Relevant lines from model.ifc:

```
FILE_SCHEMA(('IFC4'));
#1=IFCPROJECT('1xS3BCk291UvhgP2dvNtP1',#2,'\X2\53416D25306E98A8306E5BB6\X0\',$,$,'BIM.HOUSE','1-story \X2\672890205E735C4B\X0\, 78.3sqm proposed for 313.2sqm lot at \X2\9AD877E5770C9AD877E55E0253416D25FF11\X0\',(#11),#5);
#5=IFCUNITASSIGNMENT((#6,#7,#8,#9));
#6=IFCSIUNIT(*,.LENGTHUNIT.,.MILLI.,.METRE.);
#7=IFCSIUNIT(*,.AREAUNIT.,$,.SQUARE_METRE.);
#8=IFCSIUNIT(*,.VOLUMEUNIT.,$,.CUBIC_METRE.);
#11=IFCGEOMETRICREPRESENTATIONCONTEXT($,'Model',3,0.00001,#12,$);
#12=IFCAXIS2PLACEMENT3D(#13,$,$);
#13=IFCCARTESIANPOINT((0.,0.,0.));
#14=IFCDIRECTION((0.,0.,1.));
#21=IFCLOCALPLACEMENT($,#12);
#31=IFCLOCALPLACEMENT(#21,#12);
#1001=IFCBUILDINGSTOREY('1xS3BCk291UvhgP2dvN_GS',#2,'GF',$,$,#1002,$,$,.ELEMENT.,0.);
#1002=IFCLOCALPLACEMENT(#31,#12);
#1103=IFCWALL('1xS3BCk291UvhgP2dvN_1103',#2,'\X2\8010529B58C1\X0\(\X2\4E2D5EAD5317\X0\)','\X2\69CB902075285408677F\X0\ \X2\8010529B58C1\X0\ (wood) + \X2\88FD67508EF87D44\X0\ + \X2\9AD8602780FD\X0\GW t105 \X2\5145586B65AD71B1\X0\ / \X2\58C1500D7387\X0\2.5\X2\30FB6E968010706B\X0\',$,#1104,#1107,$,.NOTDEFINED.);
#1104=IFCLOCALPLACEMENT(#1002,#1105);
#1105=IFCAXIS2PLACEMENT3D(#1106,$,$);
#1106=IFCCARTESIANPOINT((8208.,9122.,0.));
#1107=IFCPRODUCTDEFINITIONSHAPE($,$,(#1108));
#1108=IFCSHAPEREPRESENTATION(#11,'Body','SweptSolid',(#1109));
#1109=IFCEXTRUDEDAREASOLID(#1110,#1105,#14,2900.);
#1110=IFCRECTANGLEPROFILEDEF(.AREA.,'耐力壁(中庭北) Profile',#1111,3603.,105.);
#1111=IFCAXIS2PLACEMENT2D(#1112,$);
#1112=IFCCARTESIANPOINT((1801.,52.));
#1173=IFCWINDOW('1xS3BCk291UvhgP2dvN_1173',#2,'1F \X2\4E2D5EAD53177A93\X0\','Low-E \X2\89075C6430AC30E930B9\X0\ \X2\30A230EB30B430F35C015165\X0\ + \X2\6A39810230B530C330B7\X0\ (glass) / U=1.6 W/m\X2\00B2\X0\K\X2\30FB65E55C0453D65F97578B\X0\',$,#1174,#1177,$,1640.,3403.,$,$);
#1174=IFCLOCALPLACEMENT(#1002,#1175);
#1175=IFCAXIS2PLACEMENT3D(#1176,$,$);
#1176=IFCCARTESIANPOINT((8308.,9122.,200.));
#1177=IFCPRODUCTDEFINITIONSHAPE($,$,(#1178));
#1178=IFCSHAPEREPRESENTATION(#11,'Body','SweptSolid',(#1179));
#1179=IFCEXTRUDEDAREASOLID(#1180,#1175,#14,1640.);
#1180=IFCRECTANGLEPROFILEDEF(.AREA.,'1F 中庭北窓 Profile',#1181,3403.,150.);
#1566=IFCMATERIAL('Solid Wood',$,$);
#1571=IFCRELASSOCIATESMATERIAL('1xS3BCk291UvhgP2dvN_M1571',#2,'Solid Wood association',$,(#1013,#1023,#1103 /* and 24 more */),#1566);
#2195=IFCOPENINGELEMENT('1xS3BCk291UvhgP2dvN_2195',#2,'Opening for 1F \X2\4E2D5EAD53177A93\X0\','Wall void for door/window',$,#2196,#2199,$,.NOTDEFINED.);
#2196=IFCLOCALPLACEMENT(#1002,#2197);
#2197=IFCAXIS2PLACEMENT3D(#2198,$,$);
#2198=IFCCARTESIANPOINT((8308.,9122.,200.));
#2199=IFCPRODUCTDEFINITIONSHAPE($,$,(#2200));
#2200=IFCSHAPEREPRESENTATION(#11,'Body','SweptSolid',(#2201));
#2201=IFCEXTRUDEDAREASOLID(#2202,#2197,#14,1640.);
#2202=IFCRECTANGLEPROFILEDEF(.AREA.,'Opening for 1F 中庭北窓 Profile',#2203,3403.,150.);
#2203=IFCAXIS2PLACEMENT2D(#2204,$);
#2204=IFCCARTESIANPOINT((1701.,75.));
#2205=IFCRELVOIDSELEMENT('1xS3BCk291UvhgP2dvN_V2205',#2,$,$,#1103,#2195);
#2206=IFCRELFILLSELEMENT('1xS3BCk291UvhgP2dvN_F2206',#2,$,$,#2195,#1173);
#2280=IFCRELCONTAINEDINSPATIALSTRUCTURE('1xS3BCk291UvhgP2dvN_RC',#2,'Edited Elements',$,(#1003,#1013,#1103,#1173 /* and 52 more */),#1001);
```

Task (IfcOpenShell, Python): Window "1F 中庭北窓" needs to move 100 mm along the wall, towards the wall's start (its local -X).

```python
import ifcopenshell
import ifcopenshell.api.geometry
import ifcopenshell.util.placement

model = ifcopenshell.open("model.ifc")

window = model.by_guid("1xS3BCk291UvhgP2dvN_1173")
opening = window.FillsVoids[0].RelatingOpeningElement
wall = opening.VoidsElements[0].RelatingBuildingElement

wall_matrix = ifcopenshell.util.placement.get_local_placement(wall.ObjectPlacement)
shift = wall_matrix[:3, 0] * -100.0
before = ifcopenshell.util.placement.get_local_placement(window.ObjectPlacement)[:3, 3].copy()

# The window is not placed relative to its opening, so move both.
for product in (opening, window):
    matrix = ifcopenshell.util.placement.get_local_placement(product.ObjectPlacement)
    matrix[:3, 3] += shift
    ifcopenshell.api.geometry.edit_object_placement(model, product=product, matrix=matrix, is_si=False)

after = ifcopenshell.util.placement.get_local_placement(window.ObjectPlacement)[:3, 3]
print("window moved by", (after - before).round(3) + 0.0)

model.write("model_updated.ifc")
```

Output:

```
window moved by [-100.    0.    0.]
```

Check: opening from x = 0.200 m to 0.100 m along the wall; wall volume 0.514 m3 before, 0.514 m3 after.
